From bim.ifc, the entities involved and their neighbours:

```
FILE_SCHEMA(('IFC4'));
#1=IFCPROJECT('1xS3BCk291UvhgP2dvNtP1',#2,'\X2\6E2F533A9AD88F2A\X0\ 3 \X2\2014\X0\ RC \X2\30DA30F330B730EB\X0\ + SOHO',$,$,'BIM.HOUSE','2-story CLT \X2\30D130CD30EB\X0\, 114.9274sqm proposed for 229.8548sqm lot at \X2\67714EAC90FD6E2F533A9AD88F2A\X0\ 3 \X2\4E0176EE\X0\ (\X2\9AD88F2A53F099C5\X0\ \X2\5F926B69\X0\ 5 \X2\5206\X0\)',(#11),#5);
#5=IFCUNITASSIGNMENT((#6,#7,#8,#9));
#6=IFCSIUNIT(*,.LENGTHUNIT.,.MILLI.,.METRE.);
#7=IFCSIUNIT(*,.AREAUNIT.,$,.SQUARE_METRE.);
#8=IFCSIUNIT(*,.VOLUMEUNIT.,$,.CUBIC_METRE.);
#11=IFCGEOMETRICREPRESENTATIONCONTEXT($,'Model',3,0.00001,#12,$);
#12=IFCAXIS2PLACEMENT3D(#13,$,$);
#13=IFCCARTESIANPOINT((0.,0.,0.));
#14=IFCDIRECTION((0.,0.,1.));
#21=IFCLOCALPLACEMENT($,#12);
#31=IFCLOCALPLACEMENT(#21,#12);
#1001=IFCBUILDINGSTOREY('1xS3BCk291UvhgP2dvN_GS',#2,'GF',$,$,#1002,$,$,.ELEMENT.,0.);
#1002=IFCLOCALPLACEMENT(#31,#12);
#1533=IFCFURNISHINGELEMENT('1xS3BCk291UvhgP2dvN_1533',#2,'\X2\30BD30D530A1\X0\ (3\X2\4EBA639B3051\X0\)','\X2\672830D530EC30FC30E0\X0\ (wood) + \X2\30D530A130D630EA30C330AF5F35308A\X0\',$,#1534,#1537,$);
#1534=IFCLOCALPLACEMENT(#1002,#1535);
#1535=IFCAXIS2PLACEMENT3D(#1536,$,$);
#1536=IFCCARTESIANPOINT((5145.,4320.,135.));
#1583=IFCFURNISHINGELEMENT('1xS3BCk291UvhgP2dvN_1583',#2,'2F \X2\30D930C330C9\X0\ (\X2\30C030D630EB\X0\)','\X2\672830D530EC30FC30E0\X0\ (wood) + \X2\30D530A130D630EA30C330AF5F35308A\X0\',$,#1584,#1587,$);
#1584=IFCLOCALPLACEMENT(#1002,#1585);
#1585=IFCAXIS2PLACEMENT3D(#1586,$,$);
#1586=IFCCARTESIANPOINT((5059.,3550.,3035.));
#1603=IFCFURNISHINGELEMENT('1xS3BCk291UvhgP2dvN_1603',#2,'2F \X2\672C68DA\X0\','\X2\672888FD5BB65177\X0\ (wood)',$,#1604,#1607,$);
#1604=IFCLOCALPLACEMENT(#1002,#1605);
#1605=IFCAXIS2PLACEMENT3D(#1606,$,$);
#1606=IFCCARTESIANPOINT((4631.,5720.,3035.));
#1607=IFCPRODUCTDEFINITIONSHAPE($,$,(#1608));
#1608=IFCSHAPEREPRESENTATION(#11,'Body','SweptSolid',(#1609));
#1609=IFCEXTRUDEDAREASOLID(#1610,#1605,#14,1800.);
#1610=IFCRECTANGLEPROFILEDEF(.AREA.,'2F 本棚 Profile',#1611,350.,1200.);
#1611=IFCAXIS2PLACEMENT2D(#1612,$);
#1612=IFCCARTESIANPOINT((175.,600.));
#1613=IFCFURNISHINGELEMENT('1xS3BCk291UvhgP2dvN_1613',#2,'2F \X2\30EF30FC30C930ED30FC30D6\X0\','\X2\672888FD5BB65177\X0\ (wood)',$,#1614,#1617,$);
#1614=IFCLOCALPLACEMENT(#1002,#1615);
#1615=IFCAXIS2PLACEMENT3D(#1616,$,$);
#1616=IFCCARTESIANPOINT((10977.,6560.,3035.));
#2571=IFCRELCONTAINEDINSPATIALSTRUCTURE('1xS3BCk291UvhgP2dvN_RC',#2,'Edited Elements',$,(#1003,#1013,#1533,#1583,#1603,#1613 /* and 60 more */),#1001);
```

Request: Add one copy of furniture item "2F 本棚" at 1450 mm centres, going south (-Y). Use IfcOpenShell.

```python
import numpy as np
import ifcopenshell
import ifcopenshell.api.geometry
import ifcopenshell.api.root
import ifcopenshell.util.element
import ifcopenshell.util.placement

model = ifcopenshell.open("bim.ifc")


def reuse_history(source, copy):
    """copy_class also copies each property set's owner history, people and application; keep the originals."""
    for rel in copy.IsDefinedBy:
        if rel.is_a("IfcRelDefinesByProperties") and (history := rel.RelatingPropertyDefinition.OwnerHistory):
            rel.RelatingPropertyDefinition.OwnerHistory = source.OwnerHistory
            ifcopenshell.util.element.remove_deep2(model, history)


source = model.by_guid("1xS3BCk291UvhgP2dvN_1603")
base = ifcopenshell.util.placement.get_local_placement(source.ObjectPlacement)
step = np.array([0.0, -1.0, 0.0]) * 1450.0

for i in range(1, 2):
    copy = ifcopenshell.api.root.copy_class(model, product=source)
    copy.Representation = ifcopenshell.util.element.copy_deep(
        model, source.Representation, exclude=["IfcGeometricRepresentationContext", "IfcRepresentationMap"]
    )
    reuse_history(source, copy)
    matrix = base.copy()
    matrix[:3, 3] += i * step
    print("added at", matrix[:3, 3].round(3) + 0.0)
    ifcopenshell.api.geometry.edit_object_placement(model, product=copy, matrix=matrix, is_si=False)

model.write("bim_edited.ifc")
```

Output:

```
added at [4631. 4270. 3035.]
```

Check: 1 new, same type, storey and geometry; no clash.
